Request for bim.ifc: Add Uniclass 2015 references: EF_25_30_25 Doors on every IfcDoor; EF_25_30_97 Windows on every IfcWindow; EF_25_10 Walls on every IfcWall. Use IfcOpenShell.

First a look at what the model holds.

```python
import ifcopenshell

model = ifcopenshell.open("bim.ifc")
print(model.schema)
print("classifications:", [c.Name for c in model.by_type("IfcClassification")])
for ifc_class in ("IfcDoor", "IfcRoof", "IfcStair", "IfcWall", "IfcWindow"):
    print(ifc_class, len(model.by_type(ifc_class)))
```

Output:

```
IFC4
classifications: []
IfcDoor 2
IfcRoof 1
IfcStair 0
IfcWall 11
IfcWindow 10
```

```python
import ifcopenshell
import ifcopenshell.api.classification

model = ifcopenshell.open("bim.ifc")

system = ifcopenshell.api.classification.add_classification(model, classification="Uniclass 2015")

codes = {
    "IfcDoor": ("EF_25_30_25", "Doors"),
    "IfcWindow": ("EF_25_30_97", "Windows"),
    "IfcWall": ("EF_25_10", "Walls"),
}
for ifc_class, (code, name) in codes.items():
    products = model.by_type(ifc_class)
    ifcopenshell.api.classification.add_reference(
        model, products=products, classification=system, identification=code, name=name
    )
    print(code, len(products))

model.write("bim_edited.ifc")
```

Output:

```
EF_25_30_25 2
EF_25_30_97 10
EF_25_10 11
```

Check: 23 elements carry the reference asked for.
